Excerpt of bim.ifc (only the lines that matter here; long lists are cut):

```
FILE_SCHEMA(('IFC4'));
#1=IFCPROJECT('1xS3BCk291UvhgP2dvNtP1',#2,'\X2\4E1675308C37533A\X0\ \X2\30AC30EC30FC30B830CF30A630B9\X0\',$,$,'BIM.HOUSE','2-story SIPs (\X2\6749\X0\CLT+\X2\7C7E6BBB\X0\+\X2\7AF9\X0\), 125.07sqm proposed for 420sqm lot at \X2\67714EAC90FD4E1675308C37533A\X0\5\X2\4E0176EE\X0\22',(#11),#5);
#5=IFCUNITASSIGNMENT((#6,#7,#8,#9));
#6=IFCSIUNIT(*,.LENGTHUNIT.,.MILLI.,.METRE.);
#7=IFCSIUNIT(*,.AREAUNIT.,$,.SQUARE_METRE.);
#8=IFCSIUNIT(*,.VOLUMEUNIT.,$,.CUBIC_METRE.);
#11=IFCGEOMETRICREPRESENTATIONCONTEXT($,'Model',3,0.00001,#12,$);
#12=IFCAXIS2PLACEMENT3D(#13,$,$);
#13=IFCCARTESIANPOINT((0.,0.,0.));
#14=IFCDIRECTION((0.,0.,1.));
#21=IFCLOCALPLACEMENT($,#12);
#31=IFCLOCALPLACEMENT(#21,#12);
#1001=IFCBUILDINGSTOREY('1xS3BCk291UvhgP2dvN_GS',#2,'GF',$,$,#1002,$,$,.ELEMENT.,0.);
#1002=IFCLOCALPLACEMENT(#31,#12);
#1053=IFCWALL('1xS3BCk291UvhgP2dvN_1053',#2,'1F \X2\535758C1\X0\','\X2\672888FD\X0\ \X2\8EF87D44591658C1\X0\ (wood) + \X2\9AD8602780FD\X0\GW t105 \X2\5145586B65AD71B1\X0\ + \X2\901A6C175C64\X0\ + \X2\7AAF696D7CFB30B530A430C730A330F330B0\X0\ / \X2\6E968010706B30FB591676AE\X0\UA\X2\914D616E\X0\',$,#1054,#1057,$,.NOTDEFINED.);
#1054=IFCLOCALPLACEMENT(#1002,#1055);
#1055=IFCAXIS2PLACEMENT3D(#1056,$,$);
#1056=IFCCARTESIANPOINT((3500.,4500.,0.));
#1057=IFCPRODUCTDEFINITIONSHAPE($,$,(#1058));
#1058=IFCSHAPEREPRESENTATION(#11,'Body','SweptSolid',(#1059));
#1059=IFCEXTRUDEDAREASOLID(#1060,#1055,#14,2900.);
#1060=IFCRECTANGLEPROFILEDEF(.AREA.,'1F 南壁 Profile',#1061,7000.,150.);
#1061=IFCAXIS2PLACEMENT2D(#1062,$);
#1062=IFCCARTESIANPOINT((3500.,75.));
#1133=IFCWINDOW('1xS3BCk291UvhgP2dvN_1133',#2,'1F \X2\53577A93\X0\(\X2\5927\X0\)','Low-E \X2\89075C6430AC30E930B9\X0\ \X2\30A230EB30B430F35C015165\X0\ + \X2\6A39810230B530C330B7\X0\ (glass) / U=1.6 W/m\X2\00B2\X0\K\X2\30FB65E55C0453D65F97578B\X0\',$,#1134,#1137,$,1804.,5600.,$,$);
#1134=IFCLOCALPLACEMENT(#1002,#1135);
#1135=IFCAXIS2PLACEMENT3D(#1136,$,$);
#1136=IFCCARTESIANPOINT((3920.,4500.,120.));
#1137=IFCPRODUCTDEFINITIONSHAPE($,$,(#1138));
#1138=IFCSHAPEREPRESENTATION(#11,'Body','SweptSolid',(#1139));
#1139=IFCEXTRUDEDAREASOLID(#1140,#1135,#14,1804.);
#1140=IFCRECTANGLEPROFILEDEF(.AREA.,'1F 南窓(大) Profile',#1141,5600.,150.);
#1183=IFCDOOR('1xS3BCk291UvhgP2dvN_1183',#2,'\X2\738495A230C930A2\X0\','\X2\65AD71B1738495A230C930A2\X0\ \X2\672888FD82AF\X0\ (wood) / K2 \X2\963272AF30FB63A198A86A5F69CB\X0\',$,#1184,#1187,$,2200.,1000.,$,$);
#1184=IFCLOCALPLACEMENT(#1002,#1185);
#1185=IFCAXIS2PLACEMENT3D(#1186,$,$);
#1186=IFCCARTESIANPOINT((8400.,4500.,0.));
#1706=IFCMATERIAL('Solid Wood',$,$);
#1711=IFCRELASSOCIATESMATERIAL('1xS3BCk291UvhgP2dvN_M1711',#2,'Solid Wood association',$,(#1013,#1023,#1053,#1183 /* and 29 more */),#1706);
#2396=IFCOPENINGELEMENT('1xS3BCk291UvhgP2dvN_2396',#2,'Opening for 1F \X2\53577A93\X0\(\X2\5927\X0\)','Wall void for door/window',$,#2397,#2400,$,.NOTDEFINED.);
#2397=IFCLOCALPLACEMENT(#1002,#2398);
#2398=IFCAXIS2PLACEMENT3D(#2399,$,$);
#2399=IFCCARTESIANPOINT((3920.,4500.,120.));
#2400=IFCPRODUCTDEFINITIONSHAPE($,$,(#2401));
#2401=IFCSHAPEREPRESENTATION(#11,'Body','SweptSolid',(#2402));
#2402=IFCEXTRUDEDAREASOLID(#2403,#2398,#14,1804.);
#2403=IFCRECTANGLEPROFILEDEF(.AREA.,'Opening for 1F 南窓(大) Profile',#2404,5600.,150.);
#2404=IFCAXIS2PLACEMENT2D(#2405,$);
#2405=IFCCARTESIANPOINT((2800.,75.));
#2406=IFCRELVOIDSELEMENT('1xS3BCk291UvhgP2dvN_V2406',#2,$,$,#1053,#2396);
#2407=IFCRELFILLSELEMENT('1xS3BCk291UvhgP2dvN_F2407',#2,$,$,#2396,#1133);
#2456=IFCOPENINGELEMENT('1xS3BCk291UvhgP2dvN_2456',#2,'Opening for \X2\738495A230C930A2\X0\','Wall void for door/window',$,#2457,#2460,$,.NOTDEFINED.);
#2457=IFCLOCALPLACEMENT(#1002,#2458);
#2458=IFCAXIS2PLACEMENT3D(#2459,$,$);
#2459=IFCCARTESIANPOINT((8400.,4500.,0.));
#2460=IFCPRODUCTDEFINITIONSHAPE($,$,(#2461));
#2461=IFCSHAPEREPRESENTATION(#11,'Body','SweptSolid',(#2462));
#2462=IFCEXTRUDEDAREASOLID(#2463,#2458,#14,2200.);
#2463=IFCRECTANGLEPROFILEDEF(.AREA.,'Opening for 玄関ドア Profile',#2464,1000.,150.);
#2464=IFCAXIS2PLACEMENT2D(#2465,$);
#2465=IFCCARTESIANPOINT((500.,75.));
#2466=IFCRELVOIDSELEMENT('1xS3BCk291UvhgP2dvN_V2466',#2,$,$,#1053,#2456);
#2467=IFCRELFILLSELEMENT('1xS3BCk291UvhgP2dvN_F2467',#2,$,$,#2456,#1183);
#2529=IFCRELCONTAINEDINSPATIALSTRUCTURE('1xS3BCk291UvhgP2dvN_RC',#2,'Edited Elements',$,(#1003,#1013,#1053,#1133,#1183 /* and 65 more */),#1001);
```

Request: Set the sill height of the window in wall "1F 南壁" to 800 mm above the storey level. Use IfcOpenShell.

```python
import numpy as np
import ifcopenshell
import ifcopenshell.api.geometry
import ifcopenshell.geom
import ifcopenshell.util.element
import ifcopenshell.util.placement
import ifcopenshell.util.shape
import ifcopenshell.util.unit

model = ifcopenshell.open("bim.ifc")
unit_scale = ifcopenshell.util.unit.calculate_unit_scale(model)

window = model.by_guid("1xS3BCk291UvhgP2dvN_1133")
opening = window.FillsVoids[0].RelatingOpeningElement
storey = ifcopenshell.util.element.get_container(window, ifc_class="IfcBuildingStorey")
level = ifcopenshell.util.placement.get_local_placement(storey.ObjectPlacement)[2, 3]

# The opening's origin need not be at the sill, so measure its lowest point.
shape = ifcopenshell.geom.create_shape(ifcopenshell.geom.settings(), opening)
bottom = ifcopenshell.util.shape.get_shape_bottom_elevation(shape, shape.geometry) / unit_scale
dz = level + 0.8 / unit_scale - bottom

shift = np.array([0.0, 0.0, dz])
# The window is not placed relative to its opening, so move both.
for product in (opening, window):
    matrix = ifcopenshell.util.placement.get_local_placement(product.ObjectPlacement)
    matrix[:3, 3] += shift
    ifcopenshell.api.geometry.edit_object_placement(model, product=product, matrix=matrix, is_si=False)

print(f"moved by {dz * unit_scale:+.3f} m")

model.write("bim_rev.ifc")
```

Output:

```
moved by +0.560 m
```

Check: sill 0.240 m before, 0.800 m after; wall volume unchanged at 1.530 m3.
